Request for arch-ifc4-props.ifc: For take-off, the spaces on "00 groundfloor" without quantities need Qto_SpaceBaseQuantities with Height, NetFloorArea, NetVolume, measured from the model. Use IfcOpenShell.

First a look at what the model holds.

```python
import ifcopenshell
import ifcopenshell.util.element
import ifcopenshell.util.unit

model = ifcopenshell.open("arch-ifc4-props.ifc")
print(model.schema)
for unit_type in ("LENGTHUNIT", "AREAUNIT", "VOLUMEUNIT"):
    print(unit_type, ifcopenshell.util.unit.calculate_unit_scale(model, unit_type))
storey = next(s for s in model.by_type("IfcBuildingStorey") if s.Name == "00 groundfloor")
spaces = [e for e in ifcopenshell.util.element.get_decomposition(storey) if e.is_a("IfcSpace")]
for e in sorted(spaces, key=lambda e: e.id()):
    print(e.id(), e.is_a(), e.Name, list(ifcopenshell.util.element.get_psets(e, qtos_only=True)), sep=" | ")
```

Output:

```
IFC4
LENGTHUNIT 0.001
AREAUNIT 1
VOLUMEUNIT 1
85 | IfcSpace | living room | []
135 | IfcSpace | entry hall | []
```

```python
import ifcopenshell
import ifcopenshell.api.pset
import ifcopenshell.geom
import ifcopenshell.util.element
import ifcopenshell.util.shape
import ifcopenshell.util.unit

model = ifcopenshell.open("arch-ifc4-props.ifc")
unit_scale = ifcopenshell.util.unit.calculate_unit_scale(model)
area_scale = ifcopenshell.util.unit.calculate_unit_scale(model, "AREAUNIT")
volume_scale = ifcopenshell.util.unit.calculate_unit_scale(model, "VOLUMEUNIT")
settings = ifcopenshell.geom.settings()

storey = next(s for s in model.by_type("IfcBuildingStorey") if s.Name == "00 groundfloor")
spaces = [e for e in ifcopenshell.util.element.get_decomposition(storey) if e.is_a("IfcSpace")]

for e in sorted(spaces, key=lambda e: e.id()):
    if ifcopenshell.util.element.get_psets(e, qtos_only=True, should_inherit=False):
        continue
    # Geometry comes back in metres, in the element's own axes.
    shape = ifcopenshell.geom.create_shape(settings, e)
    values = {
        "Height": ifcopenshell.util.shape.get_z(shape.geometry) / unit_scale,
        "NetFloorArea": ifcopenshell.util.shape.get_footprint_area(shape.geometry) / area_scale,
        "NetVolume": ifcopenshell.util.shape.get_volume(shape.geometry) / volume_scale,
    }
    qto = ifcopenshell.api.pset.add_qto(model, product=e, name="Qto_SpaceBaseQuantities")
    ifcopenshell.api.pset.edit_qto(model, qto=qto, properties=values)
    print(e.id(), {k: round(v, 3) for k, v in values.items()})

model.write("arch-ifc4-props_v2.ifc")
```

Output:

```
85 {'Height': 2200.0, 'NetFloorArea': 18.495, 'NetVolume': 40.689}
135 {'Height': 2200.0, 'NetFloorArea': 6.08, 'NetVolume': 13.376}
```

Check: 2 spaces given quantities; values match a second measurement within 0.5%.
